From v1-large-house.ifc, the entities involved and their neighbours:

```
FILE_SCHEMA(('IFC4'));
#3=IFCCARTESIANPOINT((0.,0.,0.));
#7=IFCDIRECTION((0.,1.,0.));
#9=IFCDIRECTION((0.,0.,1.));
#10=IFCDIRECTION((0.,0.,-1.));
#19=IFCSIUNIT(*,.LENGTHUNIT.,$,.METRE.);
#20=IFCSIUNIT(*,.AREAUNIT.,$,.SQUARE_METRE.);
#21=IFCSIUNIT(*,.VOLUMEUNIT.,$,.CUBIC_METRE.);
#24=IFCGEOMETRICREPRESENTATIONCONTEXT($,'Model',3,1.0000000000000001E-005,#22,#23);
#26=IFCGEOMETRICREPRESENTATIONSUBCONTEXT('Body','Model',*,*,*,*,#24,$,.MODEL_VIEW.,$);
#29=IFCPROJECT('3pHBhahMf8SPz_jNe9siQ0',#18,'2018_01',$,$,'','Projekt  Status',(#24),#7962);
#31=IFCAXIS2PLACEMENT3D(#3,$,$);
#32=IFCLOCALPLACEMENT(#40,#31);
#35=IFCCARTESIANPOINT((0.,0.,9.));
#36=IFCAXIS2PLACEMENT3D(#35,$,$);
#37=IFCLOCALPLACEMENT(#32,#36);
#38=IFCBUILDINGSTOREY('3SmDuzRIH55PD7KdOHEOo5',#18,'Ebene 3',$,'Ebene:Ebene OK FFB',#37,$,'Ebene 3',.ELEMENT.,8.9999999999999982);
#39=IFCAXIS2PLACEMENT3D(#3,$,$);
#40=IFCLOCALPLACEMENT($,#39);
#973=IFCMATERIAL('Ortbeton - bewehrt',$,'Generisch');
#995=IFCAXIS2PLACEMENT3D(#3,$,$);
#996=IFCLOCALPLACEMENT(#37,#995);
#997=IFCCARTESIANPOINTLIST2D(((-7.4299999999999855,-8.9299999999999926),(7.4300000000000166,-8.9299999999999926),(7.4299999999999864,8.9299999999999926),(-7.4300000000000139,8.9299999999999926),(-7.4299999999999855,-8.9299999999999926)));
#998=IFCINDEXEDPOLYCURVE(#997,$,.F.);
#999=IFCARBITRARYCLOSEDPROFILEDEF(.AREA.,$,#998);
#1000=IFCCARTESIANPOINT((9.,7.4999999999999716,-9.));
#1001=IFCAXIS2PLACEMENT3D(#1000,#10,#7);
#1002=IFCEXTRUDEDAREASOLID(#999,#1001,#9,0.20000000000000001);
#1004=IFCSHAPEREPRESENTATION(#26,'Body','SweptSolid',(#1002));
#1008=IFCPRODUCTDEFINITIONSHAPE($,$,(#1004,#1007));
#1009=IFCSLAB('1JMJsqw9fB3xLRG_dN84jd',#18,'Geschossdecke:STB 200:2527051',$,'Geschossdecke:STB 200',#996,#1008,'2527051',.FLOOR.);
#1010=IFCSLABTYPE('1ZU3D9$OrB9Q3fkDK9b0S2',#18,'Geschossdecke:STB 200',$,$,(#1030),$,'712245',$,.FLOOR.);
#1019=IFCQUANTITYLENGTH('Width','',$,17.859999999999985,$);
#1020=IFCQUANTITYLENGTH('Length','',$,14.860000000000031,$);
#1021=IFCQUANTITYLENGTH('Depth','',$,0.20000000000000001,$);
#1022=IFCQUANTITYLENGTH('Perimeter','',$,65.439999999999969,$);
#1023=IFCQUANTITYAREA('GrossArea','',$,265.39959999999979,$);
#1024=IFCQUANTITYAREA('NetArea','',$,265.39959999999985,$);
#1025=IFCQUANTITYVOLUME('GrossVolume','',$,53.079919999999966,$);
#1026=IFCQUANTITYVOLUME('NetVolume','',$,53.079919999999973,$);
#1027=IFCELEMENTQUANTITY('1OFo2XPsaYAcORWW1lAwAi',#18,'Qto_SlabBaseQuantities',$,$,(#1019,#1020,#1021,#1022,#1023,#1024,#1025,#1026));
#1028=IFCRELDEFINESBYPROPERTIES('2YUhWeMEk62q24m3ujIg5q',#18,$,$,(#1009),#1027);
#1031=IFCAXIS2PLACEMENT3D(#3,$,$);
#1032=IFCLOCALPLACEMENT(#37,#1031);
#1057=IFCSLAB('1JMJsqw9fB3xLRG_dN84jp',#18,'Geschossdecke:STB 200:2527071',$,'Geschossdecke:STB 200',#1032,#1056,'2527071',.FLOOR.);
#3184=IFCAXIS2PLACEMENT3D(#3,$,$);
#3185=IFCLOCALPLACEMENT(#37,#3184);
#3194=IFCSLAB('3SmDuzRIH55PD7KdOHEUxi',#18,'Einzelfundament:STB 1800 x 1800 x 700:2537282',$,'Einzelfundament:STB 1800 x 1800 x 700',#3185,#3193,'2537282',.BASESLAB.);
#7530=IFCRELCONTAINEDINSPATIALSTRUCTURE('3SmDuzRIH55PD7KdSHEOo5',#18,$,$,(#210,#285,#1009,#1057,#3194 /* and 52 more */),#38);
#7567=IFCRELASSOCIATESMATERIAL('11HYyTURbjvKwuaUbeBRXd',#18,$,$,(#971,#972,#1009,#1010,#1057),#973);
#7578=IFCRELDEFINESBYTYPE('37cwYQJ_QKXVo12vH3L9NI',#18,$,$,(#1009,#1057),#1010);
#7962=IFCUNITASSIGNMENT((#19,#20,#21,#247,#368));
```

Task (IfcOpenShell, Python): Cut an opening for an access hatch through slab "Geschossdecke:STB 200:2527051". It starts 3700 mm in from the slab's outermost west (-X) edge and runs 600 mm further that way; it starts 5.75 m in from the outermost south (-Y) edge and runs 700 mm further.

```python
import numpy as np
import ifcopenshell
import ifcopenshell.api.feature
import ifcopenshell.api.geometry
import ifcopenshell.api.pset
import ifcopenshell.api.root
import ifcopenshell.geom
import ifcopenshell.util.element
import ifcopenshell.util.placement
import ifcopenshell.util.representation
import ifcopenshell.util.shape
import ifcopenshell.util.unit

model = ifcopenshell.open("v1-large-house.ifc")
unit_scale = ifcopenshell.util.unit.calculate_unit_scale(model)
area_scale = ifcopenshell.util.unit.calculate_unit_scale(model, "AREAUNIT")
volume_scale = ifcopenshell.util.unit.calculate_unit_scale(model, "VOLUMEUNIT")
settings = ifcopenshell.geom.settings()


def volume(element):
    """Net volume in cubic metres, openings subtracted."""
    shape = ifcopenshell.geom.create_shape(settings, element)
    return ifcopenshell.util.shape.get_volume(shape.geometry)


slab = model.by_guid("1JMJsqw9fB3xLRG_dN84jd")
before = volume(slab)

# Extent in the slab's own axes, in metres. The edges named are its -X and -Y sides.
slab_shape = ifcopenshell.geom.create_shape(settings, slab)
vertices = ifcopenshell.util.shape.get_vertices(slab_shape.geometry)
x_min, y_min, bottom = vertices.min(axis=0)
top = vertices[:, 2].max()

opening = ifcopenshell.api.root.create_entity(model, ifc_class="IfcOpeningElement", name="Access hatch opening", predefined_type="OPENING")
context = ifcopenshell.util.representation.get_context(model, "Model", "Body", "MODEL_VIEW")
width, depth = 0.6, 0.7
outline = [(0.0, 0.0), (width, 0.0), (width, depth), (0.0, depth), (0.0, 0.0)]
# Overshoot both faces by 50 mm so the cut is clean.
shape = ifcopenshell.api.geometry.add_slab_representation(
    model, context=context, depth=top - bottom + 0.1, polyline=outline
)
ifcopenshell.api.geometry.assign_representation(model, product=opening, representation=shape)

matrix = ifcopenshell.util.placement.get_local_placement(slab.ObjectPlacement)
matrix[:, 3] = matrix @ np.append(np.array([x_min + 3.7, y_min + 5.75, bottom - 0.05]) / unit_scale, 1.0)
ifcopenshell.api.geometry.edit_object_placement(model, product=opening, matrix=matrix, is_si=False)
ifcopenshell.api.feature.add_feature(model, feature=opening, element=slab)

after = volume(slab)

# Update the slab's stored quantities.
qto = model.by_id(ifcopenshell.util.element.get_pset(slab, "Qto_SlabBaseQuantities", should_inherit=False)["id"])
ifcopenshell.api.pset.edit_qto(model, qto=qto, properties={
    "NetArea": after / (top - bottom) / area_scale,
    "NetVolume": after / volume_scale,
})

print(f"slab volume {before:.3f} -> {after:.3f} m3")

model.write("v1-large-house_v2.ifc")
```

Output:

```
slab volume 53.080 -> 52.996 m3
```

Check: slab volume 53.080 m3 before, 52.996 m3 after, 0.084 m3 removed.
